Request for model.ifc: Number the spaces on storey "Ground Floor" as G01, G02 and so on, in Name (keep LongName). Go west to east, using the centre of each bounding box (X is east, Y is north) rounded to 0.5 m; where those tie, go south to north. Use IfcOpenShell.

First a look at what the model holds.

```python
import ifcopenshell
import ifcopenshell.util.element
import ifcopenshell.util.placement

model = ifcopenshell.open("model.ifc")
print(model.schema)
storey = next(s for s in model.by_type("IfcBuildingStorey") if s.Name == "Ground Floor")
spaces = [e for e in ifcopenshell.util.element.get_decomposition(storey) if e.is_a("IfcSpace")]
for e in sorted(spaces, key=lambda e: e.id()):
    origin = ifcopenshell.util.placement.get_local_placement(e.ObjectPlacement)[:3, 3]
    print(e.id(), e.Name, e.LongName, origin.round(2) + 0.0, sep=" | ")
```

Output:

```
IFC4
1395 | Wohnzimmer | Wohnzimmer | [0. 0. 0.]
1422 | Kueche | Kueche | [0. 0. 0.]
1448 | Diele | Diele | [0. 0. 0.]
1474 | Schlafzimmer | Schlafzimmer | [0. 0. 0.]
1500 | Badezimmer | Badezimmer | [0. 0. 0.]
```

```python
import ifcopenshell
import ifcopenshell.geom
import ifcopenshell.util.element
import ifcopenshell.util.shape

model = ifcopenshell.open("model.ifc")
settings = ifcopenshell.geom.settings()
settings.set("use-world-coords", True)


def centre(element):
    shape = ifcopenshell.geom.create_shape(settings, element)
    return ifcopenshell.util.shape.get_bbox_centroid(shape.geometry)


storey = next(s for s in model.by_type("IfcBuildingStorey") if s.Name == "Ground Floor")
spaces = [e for e in ifcopenshell.util.element.get_decomposition(storey) if e.is_a("IfcSpace")]

# Insertion points can sit at a corner or the storey origin, so sort by the geometry (in metres).
centres = {e: centre(e) for e in spaces}
spaces.sort(key=lambda e: (round(centres[e][0] / 0.5), centres[e][1]))

for i, e in enumerate(spaces, start=1):
    number = f"G{i:02d}"
    e.Name = number
    print(e.id(), number)

model.write("model_rev.ifc")
```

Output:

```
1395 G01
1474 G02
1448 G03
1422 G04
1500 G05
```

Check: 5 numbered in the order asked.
